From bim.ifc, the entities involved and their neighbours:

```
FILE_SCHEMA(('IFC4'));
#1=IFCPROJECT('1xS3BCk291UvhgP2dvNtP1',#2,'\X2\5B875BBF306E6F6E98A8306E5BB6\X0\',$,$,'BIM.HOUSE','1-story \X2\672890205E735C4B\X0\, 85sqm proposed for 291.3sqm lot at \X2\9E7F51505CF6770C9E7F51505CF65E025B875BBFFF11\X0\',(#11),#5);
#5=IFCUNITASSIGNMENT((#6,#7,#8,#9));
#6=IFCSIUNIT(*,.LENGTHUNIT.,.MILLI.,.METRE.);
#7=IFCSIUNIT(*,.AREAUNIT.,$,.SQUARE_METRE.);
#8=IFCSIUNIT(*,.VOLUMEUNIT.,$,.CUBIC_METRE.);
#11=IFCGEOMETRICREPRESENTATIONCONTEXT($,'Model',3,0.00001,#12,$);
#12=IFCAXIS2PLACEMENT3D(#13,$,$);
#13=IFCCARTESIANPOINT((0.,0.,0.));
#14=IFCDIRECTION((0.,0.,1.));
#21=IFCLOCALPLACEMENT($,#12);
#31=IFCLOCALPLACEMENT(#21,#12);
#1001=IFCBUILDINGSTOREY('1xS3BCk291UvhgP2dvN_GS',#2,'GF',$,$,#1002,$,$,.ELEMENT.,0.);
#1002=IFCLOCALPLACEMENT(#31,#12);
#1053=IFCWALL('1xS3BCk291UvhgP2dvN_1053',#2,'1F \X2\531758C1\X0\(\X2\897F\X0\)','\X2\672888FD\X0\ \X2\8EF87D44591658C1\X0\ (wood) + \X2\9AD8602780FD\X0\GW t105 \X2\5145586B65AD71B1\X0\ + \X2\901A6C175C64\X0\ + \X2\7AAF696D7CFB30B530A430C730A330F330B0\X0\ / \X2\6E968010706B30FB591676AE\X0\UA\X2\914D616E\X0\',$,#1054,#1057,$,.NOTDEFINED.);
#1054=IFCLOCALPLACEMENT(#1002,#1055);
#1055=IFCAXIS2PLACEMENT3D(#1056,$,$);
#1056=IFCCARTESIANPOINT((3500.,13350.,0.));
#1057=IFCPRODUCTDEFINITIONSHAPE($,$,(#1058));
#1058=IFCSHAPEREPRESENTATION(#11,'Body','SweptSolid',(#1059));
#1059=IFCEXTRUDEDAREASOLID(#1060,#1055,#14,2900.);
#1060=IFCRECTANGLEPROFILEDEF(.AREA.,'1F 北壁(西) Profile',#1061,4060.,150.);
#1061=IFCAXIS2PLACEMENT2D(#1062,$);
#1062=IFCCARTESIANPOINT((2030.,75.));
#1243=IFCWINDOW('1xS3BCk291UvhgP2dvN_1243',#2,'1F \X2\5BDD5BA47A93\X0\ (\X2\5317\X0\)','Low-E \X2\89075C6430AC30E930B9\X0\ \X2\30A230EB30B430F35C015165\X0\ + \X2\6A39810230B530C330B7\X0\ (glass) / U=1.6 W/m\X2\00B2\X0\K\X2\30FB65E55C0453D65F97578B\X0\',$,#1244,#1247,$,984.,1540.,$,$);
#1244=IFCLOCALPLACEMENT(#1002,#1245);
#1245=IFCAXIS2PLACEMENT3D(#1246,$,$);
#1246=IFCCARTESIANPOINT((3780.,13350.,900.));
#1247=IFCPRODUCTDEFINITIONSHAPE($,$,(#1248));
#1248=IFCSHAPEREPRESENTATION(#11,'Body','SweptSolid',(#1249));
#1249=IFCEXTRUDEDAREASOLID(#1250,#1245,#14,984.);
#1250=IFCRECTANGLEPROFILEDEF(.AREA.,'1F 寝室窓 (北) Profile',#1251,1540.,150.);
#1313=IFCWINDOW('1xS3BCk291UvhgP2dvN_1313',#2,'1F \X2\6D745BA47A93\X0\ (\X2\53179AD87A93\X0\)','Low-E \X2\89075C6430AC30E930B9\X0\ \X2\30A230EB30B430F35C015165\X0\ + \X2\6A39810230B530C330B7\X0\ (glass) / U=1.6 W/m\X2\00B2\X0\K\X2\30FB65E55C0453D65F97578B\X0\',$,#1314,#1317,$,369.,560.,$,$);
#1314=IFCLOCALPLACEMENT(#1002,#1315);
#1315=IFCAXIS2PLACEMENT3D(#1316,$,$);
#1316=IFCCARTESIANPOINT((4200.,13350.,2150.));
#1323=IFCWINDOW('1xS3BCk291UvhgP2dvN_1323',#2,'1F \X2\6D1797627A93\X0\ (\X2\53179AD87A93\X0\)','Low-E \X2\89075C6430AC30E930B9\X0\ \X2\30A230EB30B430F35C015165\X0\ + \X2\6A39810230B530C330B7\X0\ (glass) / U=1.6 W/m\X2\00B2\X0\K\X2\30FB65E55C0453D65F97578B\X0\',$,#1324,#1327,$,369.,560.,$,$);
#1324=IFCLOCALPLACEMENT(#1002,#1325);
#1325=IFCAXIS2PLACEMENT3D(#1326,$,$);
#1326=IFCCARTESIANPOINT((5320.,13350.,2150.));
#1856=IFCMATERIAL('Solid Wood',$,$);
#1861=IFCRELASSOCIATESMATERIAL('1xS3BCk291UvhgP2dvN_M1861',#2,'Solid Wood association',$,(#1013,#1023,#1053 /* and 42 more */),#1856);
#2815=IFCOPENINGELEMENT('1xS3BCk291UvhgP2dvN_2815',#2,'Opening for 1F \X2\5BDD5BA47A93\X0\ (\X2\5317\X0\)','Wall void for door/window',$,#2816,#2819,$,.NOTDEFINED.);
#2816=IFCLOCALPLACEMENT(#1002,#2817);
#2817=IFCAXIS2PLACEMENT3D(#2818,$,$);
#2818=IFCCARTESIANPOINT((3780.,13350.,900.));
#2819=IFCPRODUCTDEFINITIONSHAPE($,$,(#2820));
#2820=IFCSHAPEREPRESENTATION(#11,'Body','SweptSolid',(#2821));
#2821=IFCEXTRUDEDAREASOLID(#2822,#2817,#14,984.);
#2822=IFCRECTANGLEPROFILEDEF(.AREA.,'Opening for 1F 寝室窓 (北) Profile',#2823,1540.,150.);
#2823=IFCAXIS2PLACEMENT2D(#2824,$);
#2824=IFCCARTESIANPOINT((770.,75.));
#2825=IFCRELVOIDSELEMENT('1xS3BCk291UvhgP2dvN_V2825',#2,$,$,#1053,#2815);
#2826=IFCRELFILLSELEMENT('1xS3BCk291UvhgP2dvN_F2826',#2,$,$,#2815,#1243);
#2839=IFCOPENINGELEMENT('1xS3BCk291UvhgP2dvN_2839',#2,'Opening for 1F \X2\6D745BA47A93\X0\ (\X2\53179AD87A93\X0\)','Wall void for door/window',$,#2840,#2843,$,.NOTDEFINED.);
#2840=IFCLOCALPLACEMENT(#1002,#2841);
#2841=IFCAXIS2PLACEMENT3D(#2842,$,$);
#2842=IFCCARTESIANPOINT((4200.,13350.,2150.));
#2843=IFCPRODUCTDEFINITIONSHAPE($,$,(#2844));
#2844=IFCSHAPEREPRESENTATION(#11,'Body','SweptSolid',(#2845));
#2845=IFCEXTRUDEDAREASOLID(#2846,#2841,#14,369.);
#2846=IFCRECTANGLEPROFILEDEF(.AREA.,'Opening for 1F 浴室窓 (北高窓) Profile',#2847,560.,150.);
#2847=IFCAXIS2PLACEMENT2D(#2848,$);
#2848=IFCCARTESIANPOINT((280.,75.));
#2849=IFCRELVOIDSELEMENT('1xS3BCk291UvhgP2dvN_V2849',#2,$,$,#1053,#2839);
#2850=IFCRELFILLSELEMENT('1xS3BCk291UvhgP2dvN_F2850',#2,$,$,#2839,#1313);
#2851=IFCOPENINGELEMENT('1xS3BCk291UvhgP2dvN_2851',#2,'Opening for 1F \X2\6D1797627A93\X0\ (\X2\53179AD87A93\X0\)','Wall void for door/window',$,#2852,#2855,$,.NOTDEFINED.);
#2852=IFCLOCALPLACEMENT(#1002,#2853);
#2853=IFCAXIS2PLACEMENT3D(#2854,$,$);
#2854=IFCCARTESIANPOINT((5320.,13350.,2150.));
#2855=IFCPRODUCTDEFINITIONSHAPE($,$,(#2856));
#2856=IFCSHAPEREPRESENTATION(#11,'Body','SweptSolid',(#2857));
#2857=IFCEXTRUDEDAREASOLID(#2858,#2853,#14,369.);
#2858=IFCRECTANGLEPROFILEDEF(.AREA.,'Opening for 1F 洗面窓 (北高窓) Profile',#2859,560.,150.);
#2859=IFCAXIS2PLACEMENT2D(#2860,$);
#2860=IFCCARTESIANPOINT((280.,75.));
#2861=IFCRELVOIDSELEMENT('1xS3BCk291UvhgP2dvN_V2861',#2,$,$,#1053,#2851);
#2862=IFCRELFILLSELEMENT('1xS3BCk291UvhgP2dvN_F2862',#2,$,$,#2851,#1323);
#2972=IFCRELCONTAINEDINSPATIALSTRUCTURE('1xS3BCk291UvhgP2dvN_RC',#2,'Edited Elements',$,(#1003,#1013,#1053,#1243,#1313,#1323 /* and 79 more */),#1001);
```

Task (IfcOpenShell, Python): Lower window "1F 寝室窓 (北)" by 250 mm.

```python
import numpy as np
import ifcopenshell
import ifcopenshell.api.geometry
import ifcopenshell.util.placement
import ifcopenshell.util.unit

model = ifcopenshell.open("bim.ifc")
unit_scale = ifcopenshell.util.unit.calculate_unit_scale(model)

window = model.by_guid("1xS3BCk291UvhgP2dvN_1243")
opening = window.FillsVoids[0].RelatingOpeningElement
dz = -250.0

shift = np.array([0.0, 0.0, dz])
# The window is not placed relative to its opening, so move both.
for product in (opening, window):
    matrix = ifcopenshell.util.placement.get_local_placement(product.ObjectPlacement)
    matrix[:3, 3] += shift
    ifcopenshell.api.geometry.edit_object_placement(model, product=product, matrix=matrix, is_si=False)

print(f"moved by {dz * unit_scale:+.3f} m")

model.write("bim_edited.ifc")
```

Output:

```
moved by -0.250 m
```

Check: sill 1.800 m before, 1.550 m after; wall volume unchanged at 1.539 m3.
